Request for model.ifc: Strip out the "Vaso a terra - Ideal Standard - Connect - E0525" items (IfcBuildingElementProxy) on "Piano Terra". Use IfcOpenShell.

First a look at what the model holds.

```python
import ifcopenshell
import ifcopenshell.util.element

model = ifcopenshell.open("model.ifc")
print(model.schema)
storey = next(s for s in model.by_type("IfcBuildingStorey") if s.Name == "Piano Terra")
proxies = [e for e in ifcopenshell.util.element.get_decomposition(storey) if e.is_a("IfcBuildingElementProxy")]
seen = {}
for e in proxies:
    element_type = ifcopenshell.util.element.get_type(e)
    name = element_type.Name if element_type not in (None, e) else None
    seen[name] = seen.get(name, 0) + 1
for name, count in sorted(seen.items(), key=str):
    print(count, "x", name)
```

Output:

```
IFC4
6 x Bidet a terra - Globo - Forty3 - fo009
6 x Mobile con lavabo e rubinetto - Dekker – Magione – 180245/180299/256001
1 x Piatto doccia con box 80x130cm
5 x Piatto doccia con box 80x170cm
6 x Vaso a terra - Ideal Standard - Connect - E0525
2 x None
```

```python
import ifcopenshell
import ifcopenshell.api.root
import ifcopenshell.util.element

model = ifcopenshell.open("model.ifc")

storey = next(s for s in model.by_type("IfcBuildingStorey") if s.Name == "Piano Terra")
proxies = [e for e in ifcopenshell.util.element.get_decomposition(storey) if e.is_a("IfcBuildingElementProxy")]
targets = [e for e in proxies if (t := ifcopenshell.util.element.get_type(e)) not in (None, e) and t.Name == "Vaso a terra - Ideal Standard - Connect - E0525"]

for e in targets:
    ifcopenshell.api.root.remove_product(model, product=e)
print(len(targets), "removed")

model.write("model_v2.ifc")
```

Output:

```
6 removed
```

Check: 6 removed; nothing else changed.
